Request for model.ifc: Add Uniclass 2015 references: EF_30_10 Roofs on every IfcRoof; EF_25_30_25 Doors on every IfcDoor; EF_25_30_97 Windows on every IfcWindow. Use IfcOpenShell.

First a look at what the model holds.

```python
import ifcopenshell

model = ifcopenshell.open("model.ifc")
print(model.schema)
print("classifications:", [c.Name for c in model.by_type("IfcClassification")])
for ifc_class in ("IfcDoor", "IfcRoof", "IfcStair", "IfcWall", "IfcWindow"):
    print(ifc_class, len(model.by_type(ifc_class)))
```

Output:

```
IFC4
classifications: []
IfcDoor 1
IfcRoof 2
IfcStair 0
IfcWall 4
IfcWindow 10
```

```python
import ifcopenshell
import ifcopenshell.api.classification

model = ifcopenshell.open("model.ifc")

system = ifcopenshell.api.classification.add_classification(model, classification="Uniclass 2015")

codes = {
    "IfcRoof": ("EF_30_10", "Roofs"),
    "IfcDoor": ("EF_25_30_25", "Doors"),
    "IfcWindow": ("EF_25_30_97", "Windows"),
}
for ifc_class, (code, name) in codes.items():
    products = model.by_type(ifc_class)
    ifcopenshell.api.classification.add_reference(
        model, products=products, classification=system, identification=code, name=name
    )
    print(code, len(products))

model.write("model_rev.ifc")
```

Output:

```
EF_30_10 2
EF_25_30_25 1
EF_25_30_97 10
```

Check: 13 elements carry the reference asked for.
